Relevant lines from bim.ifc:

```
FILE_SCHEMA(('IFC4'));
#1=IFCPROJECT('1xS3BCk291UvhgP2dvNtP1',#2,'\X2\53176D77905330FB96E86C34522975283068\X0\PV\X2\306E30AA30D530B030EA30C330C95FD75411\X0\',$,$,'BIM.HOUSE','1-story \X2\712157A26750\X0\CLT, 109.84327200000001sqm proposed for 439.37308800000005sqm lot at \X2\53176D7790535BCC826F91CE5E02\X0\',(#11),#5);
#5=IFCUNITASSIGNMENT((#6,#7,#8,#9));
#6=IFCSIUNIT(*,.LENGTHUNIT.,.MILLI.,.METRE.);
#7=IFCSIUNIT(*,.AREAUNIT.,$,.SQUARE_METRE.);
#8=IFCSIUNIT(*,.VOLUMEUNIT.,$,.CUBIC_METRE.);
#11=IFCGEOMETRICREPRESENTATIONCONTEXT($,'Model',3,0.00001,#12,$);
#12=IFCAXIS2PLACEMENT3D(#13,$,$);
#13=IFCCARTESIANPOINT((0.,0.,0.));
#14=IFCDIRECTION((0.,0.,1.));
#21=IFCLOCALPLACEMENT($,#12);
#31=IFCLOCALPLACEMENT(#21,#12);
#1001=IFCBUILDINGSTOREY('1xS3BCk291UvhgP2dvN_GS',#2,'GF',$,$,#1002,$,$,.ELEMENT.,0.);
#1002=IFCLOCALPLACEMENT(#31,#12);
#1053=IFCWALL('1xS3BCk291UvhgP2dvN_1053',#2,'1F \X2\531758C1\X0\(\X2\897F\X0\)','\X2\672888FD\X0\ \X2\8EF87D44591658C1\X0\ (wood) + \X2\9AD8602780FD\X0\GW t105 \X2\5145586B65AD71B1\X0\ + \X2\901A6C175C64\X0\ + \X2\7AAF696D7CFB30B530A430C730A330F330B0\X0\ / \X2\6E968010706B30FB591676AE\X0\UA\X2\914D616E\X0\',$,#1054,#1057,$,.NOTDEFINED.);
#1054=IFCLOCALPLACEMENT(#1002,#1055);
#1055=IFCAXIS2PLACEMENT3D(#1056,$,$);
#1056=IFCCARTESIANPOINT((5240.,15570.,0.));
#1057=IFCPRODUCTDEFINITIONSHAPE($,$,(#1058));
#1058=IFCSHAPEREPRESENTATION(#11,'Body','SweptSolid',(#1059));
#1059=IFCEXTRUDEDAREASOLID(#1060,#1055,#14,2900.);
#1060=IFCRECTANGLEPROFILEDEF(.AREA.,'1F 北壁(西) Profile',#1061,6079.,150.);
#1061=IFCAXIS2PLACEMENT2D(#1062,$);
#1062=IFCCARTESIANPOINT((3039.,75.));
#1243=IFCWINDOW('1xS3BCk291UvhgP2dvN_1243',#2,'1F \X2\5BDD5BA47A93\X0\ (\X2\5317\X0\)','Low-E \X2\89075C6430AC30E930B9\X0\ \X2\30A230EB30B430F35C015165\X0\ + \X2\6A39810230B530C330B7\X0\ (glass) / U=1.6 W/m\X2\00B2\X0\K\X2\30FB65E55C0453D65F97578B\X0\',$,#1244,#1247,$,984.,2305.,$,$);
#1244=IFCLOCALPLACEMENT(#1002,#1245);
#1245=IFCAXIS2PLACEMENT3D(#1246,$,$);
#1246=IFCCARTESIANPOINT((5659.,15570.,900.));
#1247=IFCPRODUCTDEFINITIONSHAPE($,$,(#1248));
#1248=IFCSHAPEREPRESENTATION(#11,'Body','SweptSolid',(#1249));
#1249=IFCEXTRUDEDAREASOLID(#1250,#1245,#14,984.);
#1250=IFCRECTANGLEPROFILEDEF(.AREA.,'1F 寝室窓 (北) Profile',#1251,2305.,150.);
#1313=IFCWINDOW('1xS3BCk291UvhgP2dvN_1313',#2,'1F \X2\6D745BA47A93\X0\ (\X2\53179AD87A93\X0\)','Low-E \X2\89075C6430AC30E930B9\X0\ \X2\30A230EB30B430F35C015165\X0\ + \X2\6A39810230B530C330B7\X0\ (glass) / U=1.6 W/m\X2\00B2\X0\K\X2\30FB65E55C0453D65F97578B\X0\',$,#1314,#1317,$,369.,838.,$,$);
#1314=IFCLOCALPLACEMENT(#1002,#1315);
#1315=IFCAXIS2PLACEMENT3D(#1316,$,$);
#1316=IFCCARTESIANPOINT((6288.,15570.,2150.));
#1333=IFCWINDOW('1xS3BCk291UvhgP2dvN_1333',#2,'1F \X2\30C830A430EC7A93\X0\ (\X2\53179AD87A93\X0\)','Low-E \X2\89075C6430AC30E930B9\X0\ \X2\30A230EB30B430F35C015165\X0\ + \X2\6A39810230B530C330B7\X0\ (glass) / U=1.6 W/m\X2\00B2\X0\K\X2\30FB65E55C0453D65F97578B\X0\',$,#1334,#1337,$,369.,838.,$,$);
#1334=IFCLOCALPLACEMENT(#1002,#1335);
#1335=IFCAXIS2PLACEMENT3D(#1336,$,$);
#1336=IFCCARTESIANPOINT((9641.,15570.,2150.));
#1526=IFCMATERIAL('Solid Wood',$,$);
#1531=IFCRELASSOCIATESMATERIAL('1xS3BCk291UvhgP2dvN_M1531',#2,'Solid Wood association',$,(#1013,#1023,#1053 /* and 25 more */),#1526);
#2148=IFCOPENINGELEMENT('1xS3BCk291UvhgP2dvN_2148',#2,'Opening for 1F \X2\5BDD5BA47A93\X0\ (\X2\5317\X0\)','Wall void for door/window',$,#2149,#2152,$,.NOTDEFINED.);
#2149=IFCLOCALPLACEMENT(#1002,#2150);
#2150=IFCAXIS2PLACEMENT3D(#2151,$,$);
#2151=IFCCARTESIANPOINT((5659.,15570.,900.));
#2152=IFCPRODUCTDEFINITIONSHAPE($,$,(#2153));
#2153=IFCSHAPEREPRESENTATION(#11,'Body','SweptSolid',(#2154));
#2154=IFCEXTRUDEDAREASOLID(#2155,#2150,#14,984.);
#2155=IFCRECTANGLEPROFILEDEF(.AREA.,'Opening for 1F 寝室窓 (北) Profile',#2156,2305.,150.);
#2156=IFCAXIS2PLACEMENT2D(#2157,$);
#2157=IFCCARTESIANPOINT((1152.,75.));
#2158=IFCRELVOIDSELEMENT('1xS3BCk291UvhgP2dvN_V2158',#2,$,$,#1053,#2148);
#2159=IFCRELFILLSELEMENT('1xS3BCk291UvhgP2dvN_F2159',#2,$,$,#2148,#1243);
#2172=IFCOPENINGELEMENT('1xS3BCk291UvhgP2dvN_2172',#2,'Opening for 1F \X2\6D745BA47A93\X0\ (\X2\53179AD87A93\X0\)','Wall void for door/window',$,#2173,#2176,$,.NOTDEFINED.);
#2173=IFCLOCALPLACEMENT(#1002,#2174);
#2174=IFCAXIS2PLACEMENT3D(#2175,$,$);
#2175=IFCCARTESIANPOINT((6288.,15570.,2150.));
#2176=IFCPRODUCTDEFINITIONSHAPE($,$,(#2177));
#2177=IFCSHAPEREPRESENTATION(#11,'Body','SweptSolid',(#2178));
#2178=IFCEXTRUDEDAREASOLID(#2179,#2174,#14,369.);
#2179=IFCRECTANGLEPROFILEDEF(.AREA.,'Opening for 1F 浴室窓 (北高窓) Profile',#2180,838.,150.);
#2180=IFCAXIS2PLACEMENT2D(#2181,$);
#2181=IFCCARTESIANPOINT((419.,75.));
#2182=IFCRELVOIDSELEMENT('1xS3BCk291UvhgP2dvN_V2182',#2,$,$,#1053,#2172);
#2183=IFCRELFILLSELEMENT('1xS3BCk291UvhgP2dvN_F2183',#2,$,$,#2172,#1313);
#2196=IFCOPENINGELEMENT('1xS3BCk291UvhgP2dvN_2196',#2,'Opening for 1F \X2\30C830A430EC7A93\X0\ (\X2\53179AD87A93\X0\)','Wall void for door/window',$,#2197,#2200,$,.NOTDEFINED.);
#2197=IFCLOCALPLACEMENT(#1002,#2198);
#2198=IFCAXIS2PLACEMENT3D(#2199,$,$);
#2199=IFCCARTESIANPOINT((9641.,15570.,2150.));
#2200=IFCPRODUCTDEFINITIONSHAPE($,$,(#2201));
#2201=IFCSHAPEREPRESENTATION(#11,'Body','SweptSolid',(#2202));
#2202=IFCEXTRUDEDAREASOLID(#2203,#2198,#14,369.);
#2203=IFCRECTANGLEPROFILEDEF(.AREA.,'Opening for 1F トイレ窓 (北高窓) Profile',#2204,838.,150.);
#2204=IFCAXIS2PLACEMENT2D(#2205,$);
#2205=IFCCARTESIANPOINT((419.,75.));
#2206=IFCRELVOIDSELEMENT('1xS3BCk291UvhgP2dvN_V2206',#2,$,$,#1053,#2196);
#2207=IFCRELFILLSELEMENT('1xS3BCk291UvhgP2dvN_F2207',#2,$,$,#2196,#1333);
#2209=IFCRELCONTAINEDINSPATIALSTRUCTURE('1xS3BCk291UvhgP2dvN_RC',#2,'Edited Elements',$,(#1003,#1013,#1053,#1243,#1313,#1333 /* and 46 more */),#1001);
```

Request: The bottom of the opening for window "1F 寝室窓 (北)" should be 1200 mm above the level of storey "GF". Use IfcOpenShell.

```python
import numpy as np
import ifcopenshell
import ifcopenshell.api.geometry
import ifcopenshell.geom
import ifcopenshell.util.element
import ifcopenshell.util.placement
import ifcopenshell.util.shape
import ifcopenshell.util.unit

model = ifcopenshell.open("bim.ifc")
unit_scale = ifcopenshell.util.unit.calculate_unit_scale(model)

window = model.by_guid("1xS3BCk291UvhgP2dvN_1243")
opening = window.FillsVoids[0].RelatingOpeningElement
storey = ifcopenshell.util.element.get_container(window, ifc_class="IfcBuildingStorey")
level = ifcopenshell.util.placement.get_local_placement(storey.ObjectPlacement)[2, 3]

# The opening's origin need not be at the sill, so measure its lowest point.
shape = ifcopenshell.geom.create_shape(ifcopenshell.geom.settings(), opening)
bottom = ifcopenshell.util.shape.get_shape_bottom_elevation(shape, shape.geometry) / unit_scale
dz = level + 1.2 / unit_scale - bottom

shift = np.array([0.0, 0.0, dz])
# The window is not placed relative to its opening, so move both.
for product in (opening, window):
    matrix = ifcopenshell.util.placement.get_local_placement(product.ObjectPlacement)
    matrix[:3, 3] += shift
    ifcopenshell.api.geometry.edit_object_placement(model, product=product, matrix=matrix, is_si=False)

print(f"moved by {dz * unit_scale:+.3f} m")

model.write("bim-out.ifc")
```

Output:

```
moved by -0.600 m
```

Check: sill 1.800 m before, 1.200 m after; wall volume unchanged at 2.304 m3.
